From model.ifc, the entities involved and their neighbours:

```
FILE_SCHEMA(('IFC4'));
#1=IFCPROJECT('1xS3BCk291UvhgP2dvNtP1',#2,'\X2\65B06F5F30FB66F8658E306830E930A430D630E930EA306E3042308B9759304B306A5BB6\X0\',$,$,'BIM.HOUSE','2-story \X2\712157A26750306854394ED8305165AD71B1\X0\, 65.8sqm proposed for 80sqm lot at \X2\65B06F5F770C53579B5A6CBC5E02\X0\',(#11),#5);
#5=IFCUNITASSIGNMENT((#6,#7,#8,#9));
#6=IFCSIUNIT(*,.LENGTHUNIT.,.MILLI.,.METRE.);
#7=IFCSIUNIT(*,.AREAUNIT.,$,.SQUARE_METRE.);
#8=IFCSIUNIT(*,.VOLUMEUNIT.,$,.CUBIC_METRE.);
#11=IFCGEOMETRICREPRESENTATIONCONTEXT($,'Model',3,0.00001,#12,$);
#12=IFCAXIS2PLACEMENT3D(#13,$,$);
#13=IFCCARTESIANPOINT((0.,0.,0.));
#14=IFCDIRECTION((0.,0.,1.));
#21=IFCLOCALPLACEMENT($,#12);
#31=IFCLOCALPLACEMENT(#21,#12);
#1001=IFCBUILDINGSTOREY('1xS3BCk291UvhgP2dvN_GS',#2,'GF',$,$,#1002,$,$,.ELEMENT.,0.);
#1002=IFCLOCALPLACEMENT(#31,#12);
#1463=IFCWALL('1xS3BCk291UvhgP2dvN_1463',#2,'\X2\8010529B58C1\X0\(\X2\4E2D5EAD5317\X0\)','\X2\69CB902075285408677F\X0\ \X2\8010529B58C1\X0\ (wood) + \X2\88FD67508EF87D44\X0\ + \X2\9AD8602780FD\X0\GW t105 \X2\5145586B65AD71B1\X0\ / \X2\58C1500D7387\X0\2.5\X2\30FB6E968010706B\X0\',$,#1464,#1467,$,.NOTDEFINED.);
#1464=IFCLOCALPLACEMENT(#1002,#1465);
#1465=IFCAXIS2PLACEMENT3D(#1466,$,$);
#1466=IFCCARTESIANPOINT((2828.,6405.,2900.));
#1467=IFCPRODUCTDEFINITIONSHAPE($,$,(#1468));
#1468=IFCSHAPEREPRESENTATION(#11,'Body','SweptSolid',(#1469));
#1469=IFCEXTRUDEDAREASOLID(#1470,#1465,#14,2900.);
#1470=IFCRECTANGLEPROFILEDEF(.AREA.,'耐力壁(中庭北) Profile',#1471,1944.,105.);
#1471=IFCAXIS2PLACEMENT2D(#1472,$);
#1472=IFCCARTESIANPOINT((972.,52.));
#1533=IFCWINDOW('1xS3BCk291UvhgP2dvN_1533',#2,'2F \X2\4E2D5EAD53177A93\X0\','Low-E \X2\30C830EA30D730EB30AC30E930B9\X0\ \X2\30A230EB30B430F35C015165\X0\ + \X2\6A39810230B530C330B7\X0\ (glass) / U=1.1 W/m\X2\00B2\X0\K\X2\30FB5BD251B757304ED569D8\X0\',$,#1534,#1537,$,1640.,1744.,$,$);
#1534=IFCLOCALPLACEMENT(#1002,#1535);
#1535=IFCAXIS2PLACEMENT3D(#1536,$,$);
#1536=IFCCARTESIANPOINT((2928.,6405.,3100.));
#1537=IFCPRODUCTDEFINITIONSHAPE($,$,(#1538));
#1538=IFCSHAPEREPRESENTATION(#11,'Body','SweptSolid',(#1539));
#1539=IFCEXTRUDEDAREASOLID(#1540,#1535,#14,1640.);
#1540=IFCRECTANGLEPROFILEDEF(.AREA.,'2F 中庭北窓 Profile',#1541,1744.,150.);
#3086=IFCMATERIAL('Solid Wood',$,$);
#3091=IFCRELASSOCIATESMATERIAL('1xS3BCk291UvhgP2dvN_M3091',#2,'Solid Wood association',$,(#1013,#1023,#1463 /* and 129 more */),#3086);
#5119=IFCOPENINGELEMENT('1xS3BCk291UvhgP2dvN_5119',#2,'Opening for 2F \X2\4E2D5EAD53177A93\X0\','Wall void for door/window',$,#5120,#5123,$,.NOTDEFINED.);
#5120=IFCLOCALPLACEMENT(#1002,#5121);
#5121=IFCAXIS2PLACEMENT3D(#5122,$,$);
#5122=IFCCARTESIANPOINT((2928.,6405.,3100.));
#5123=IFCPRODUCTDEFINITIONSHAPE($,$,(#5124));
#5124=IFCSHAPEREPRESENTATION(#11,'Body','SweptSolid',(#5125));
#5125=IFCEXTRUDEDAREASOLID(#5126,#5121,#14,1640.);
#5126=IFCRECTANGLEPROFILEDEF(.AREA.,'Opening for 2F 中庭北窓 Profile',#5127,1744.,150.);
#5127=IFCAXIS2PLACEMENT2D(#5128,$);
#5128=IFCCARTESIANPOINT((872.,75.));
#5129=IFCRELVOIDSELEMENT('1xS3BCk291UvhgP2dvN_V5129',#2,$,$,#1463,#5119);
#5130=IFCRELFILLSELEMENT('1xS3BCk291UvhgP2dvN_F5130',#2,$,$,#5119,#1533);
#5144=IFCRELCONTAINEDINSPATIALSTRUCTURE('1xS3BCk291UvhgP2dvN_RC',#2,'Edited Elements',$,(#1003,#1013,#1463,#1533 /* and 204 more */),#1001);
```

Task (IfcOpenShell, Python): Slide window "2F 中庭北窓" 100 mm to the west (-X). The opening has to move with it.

```python
import ifcopenshell
import ifcopenshell.api.geometry
import ifcopenshell.util.placement
import ifcopenshell.util.unit

model = ifcopenshell.open("model.ifc")
unit_scale = ifcopenshell.util.unit.calculate_unit_scale(model)

window = model.by_guid("1xS3BCk291UvhgP2dvN_1533")
opening = window.FillsVoids[0].RelatingOpeningElement
wall = opening.VoidsElements[0].RelatingBuildingElement

wall_matrix = ifcopenshell.util.placement.get_local_placement(wall.ObjectPlacement)
shift = wall_matrix[:3, 0] * -0.1 / unit_scale
before = ifcopenshell.util.placement.get_local_placement(window.ObjectPlacement)[:3, 3].copy()

# The window is not placed relative to its opening, so move both.
for product in (opening, window):
    matrix = ifcopenshell.util.placement.get_local_placement(product.ObjectPlacement)
    matrix[:3, 3] += shift
    ifcopenshell.api.geometry.edit_object_placement(model, product=product, matrix=matrix, is_si=False)

after = ifcopenshell.util.placement.get_local_placement(window.ObjectPlacement)[:3, 3]
print("window moved by", (after - before).round(3) + 0.0)

model.write("model_edited.ifc")
```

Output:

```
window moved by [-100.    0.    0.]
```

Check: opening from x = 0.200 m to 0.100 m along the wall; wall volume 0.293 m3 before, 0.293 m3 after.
